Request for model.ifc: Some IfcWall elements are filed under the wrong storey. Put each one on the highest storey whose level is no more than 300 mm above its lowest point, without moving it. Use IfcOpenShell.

First a look at what the model holds.

```python
import ifcopenshell
import ifcopenshell.util.element
import ifcopenshell.util.placement

model = ifcopenshell.open("model.ifc")
print(model.schema)
for storey in model.by_type("IfcBuildingStorey"):
    level = ifcopenshell.util.placement.get_storey_elevation(storey)
    count = sum(e.is_a("IfcWall") for e in ifcopenshell.util.element.get_contained(storey))
    print(storey.id(), storey.Name, round(level, 3), count, sep=" | ")
```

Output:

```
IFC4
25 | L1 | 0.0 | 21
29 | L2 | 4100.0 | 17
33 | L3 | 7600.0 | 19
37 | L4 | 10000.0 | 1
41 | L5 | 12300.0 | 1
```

```python
import ifcopenshell
import ifcopenshell.api.spatial
import ifcopenshell.geom
import ifcopenshell.util.element
import ifcopenshell.util.placement
import ifcopenshell.util.shape
import ifcopenshell.util.unit

model = ifcopenshell.open("model.ifc")
unit_scale = ifcopenshell.util.unit.calculate_unit_scale(model)
settings = ifcopenshell.geom.settings()

levels = sorted(
    ((ifcopenshell.util.placement.get_storey_elevation(s) * unit_scale, s) for s in model.by_type("IfcBuildingStorey")),
    key=lambda pair: pair[0],
)

for e in model.by_type("IfcWall"):
    current = e.ContainedInStructure[0].RelatingStructure if e.ContainedInStructure else None
    if current is None or not current.is_a("IfcBuildingStorey"):
        continue
    shape = ifcopenshell.geom.create_shape(settings, e)
    bottom = ifcopenshell.util.shape.get_shape_bottom_elevation(shape, shape.geometry)
    below = [s for level, s in levels if level <= bottom + 0.3]
    storey = below[-1] if below else levels[0][1]
    if storey != current:
        # assign_container keeps the world position.
        ifcopenshell.api.spatial.assign_container(model, products=[e], relating_structure=storey)
        print(e.id(), current.Name, "->", storey.Name)

model.write("model_rev.ifc")
```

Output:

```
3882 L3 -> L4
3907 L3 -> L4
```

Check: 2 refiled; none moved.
